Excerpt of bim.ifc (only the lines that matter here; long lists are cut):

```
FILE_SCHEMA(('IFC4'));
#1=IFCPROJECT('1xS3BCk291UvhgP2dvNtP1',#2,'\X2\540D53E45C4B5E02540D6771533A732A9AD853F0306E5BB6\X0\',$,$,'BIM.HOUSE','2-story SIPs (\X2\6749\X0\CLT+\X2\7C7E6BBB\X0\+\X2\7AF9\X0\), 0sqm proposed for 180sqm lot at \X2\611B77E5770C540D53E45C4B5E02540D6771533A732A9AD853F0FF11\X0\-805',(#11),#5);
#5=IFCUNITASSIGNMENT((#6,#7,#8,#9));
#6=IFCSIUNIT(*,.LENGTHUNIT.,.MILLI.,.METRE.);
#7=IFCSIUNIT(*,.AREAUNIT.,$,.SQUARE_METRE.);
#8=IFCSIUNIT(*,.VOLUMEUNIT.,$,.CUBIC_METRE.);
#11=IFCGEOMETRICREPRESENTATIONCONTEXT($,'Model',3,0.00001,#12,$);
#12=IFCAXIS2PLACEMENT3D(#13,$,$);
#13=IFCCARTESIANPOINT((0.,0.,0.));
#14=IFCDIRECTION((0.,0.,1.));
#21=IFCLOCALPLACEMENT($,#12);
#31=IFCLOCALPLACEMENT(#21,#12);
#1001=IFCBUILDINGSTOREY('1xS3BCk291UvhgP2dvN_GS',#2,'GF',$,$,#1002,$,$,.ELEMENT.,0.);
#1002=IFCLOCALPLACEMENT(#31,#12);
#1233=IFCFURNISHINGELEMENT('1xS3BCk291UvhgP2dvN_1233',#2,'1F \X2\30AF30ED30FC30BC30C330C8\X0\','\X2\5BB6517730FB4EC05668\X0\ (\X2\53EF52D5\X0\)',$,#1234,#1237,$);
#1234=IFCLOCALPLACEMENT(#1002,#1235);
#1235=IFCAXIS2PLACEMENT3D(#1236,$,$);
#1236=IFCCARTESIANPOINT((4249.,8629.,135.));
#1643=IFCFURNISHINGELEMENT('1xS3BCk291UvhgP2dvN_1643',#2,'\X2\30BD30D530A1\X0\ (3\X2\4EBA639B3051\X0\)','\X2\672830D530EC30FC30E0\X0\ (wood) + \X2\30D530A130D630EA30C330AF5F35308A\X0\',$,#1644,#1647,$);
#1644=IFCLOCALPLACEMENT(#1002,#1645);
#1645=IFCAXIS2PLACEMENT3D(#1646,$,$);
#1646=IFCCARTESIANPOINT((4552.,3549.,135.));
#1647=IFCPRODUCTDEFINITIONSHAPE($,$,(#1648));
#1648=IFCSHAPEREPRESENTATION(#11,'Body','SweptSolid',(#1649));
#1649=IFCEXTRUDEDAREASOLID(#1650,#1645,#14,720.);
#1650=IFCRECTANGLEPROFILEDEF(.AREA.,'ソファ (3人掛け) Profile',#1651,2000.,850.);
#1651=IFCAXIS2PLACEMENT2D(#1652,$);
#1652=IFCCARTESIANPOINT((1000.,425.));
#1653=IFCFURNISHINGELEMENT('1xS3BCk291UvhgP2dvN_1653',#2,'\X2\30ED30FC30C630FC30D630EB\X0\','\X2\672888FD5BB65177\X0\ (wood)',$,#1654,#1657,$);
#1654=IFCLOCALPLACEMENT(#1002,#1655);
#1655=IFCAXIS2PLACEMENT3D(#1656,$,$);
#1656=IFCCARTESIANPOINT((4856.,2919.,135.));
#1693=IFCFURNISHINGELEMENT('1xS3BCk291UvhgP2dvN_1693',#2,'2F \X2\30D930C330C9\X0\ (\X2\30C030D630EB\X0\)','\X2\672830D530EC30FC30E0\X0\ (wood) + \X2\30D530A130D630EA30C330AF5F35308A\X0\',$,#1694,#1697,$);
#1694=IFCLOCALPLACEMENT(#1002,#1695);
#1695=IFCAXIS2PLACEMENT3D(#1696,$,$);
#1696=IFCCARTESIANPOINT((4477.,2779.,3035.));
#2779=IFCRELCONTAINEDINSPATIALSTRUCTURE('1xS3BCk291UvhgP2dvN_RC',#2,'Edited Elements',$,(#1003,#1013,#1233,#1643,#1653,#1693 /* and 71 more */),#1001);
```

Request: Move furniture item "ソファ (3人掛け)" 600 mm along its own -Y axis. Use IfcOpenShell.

```python
import ifcopenshell
import ifcopenshell.api.geometry
import ifcopenshell.util.placement
import ifcopenshell.util.unit

model = ifcopenshell.open("bim.ifc")
unit_scale = ifcopenshell.util.unit.calculate_unit_scale(model)

item = model.by_guid("1xS3BCk291UvhgP2dvN_1643")
matrix = ifcopenshell.util.placement.get_local_placement(item.ObjectPlacement)
matrix[:3, 3] -= matrix[:3, 1] * 0.6 / unit_scale
ifcopenshell.api.geometry.edit_object_placement(model, product=item, matrix=matrix, is_si=False)

print(ifcopenshell.util.placement.get_local_placement(item.ObjectPlacement).round(3) + 0.0)

model.write("bim-out.ifc")
```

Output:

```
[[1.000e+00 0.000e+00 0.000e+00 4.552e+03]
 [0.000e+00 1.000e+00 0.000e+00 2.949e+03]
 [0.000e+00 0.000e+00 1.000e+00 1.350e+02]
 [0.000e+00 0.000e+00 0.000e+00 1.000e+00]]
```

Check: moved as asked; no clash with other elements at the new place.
